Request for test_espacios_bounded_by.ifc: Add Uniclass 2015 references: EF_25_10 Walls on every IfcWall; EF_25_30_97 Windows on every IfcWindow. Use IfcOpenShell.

First a look at what the model holds.

```python
import ifcopenshell

model = ifcopenshell.open("test_espacios_bounded_by.ifc")
print(model.schema)
print("classifications:", [c.Name for c in model.by_type("IfcClassification")])
for ifc_class in ("IfcDoor", "IfcRoof", "IfcStair", "IfcWall", "IfcWindow"):
    print(ifc_class, len(model.by_type(ifc_class)))
```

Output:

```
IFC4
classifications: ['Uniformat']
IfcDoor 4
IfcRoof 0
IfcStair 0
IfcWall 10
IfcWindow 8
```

```python
import ifcopenshell
import ifcopenshell.api.classification

model = ifcopenshell.open("test_espacios_bounded_by.ifc")

system = ifcopenshell.api.classification.add_classification(model, classification="Uniclass 2015")

codes = {
    "IfcWall": ("EF_25_10", "Walls"),
    "IfcWindow": ("EF_25_30_97", "Windows"),
}
for ifc_class, (code, name) in codes.items():
    products = model.by_type(ifc_class)
    ifcopenshell.api.classification.add_reference(
        model, products=products, classification=system, identification=code, name=name
    )
    print(code, len(products))

model.write("test_espacios_bounded_by-out.ifc")
```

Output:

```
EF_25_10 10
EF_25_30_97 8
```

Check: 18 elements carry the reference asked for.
